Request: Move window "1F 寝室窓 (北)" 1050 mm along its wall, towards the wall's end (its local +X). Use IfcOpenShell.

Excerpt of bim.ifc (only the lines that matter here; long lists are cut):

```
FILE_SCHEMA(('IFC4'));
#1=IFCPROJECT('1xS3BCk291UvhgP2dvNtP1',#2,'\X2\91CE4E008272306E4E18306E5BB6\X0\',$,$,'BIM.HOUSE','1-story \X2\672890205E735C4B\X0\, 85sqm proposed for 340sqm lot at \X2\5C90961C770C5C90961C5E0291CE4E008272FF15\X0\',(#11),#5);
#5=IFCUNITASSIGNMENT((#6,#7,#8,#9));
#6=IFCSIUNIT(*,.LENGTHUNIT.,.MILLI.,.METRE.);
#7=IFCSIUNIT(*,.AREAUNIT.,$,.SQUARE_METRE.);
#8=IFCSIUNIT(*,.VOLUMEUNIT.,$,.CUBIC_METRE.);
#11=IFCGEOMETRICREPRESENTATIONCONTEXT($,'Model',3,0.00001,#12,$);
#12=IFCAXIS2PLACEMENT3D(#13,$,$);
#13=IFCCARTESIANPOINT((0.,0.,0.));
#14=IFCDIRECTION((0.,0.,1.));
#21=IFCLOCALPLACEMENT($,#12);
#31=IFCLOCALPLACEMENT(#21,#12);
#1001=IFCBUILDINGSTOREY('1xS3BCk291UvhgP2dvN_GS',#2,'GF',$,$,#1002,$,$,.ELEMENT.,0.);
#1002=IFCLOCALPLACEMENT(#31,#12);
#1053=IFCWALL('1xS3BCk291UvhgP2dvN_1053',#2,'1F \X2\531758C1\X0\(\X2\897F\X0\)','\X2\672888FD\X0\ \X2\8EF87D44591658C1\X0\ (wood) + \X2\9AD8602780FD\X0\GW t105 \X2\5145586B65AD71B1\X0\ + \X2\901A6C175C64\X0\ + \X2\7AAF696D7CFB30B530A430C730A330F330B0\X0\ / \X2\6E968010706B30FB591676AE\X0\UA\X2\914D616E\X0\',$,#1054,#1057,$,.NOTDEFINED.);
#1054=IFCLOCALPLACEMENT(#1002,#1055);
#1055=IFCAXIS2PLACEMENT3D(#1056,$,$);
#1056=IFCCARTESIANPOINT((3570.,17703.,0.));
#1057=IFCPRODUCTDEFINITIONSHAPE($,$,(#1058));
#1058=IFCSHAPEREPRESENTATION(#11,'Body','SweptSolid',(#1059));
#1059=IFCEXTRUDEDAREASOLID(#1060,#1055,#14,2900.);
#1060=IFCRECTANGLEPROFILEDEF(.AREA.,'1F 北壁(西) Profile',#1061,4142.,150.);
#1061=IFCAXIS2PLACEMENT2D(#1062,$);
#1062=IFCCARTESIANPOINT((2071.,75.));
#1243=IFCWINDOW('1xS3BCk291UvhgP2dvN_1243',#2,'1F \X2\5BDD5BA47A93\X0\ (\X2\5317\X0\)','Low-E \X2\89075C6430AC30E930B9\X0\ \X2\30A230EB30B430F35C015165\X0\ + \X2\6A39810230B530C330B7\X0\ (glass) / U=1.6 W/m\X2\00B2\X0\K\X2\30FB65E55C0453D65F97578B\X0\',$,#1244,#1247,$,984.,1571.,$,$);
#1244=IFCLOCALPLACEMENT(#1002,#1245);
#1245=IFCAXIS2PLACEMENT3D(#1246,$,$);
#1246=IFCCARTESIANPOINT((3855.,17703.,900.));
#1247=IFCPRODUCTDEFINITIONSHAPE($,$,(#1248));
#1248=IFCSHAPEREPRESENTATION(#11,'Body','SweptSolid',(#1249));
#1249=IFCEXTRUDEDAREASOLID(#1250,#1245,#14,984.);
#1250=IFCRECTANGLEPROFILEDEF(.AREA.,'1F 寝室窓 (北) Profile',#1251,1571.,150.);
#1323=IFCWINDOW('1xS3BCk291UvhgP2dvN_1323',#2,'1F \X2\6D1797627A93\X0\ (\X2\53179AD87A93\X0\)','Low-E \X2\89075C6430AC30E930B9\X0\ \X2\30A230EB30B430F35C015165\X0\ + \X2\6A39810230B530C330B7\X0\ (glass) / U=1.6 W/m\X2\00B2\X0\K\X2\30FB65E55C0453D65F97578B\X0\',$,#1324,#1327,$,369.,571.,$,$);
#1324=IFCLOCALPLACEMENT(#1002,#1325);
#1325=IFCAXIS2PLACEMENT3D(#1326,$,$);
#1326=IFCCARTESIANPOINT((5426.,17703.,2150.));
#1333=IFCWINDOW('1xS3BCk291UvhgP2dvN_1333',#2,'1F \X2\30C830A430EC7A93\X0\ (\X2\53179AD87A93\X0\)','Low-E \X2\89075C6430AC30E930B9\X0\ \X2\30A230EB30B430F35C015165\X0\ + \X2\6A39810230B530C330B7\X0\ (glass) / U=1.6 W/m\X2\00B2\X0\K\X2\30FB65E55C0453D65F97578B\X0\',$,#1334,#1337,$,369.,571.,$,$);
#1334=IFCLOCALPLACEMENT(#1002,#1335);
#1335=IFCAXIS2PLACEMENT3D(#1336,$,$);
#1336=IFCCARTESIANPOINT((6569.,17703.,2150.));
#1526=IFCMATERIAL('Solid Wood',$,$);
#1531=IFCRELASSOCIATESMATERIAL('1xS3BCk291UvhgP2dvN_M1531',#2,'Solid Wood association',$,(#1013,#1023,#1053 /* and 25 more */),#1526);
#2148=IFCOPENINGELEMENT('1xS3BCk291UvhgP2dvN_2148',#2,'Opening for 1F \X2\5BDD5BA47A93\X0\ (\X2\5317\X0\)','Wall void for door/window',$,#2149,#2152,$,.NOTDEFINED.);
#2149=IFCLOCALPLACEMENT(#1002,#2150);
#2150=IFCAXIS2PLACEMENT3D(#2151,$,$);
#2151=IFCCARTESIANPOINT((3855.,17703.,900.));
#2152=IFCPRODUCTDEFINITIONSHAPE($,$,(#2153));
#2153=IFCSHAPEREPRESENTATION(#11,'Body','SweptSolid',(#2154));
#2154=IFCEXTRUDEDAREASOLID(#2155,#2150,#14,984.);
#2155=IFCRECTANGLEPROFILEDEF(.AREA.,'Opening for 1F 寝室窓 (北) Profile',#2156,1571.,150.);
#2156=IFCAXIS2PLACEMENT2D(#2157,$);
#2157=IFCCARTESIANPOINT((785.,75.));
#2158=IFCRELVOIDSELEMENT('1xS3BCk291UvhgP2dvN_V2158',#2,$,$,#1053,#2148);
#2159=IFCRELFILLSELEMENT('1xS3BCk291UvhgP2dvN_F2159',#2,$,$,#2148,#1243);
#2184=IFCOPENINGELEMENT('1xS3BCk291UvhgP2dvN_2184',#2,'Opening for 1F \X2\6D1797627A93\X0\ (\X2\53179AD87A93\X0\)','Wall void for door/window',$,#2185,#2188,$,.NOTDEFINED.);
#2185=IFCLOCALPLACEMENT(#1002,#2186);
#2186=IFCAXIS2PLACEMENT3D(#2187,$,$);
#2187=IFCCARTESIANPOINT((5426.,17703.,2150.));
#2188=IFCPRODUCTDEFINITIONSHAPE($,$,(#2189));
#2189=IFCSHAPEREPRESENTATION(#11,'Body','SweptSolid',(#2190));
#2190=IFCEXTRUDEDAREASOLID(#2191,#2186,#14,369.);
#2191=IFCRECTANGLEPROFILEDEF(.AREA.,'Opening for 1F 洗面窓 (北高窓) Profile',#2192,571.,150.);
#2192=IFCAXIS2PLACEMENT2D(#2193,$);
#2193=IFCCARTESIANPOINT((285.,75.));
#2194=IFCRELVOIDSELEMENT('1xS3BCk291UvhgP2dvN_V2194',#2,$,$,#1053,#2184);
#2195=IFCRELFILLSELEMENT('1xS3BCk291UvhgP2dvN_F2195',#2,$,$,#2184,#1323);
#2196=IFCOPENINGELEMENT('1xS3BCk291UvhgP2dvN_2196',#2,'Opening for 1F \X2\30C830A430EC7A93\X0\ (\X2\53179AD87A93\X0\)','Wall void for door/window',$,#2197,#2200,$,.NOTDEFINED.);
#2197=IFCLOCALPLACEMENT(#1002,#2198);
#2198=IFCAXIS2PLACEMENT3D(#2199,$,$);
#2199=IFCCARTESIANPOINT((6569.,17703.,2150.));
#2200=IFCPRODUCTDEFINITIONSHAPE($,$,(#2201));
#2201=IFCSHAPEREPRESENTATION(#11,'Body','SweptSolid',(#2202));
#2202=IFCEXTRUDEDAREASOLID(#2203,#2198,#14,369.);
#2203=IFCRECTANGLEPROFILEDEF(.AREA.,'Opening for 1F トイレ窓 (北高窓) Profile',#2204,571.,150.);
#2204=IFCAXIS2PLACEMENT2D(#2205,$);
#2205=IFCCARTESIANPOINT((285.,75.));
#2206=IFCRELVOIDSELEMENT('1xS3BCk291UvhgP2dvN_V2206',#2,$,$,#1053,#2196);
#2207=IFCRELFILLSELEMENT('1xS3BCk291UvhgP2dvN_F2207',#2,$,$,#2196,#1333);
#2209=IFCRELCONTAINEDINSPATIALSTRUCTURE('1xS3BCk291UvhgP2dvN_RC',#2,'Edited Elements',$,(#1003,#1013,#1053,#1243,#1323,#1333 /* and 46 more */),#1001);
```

```python
import ifcopenshell
import ifcopenshell.api.geometry
import ifcopenshell.util.placement
import ifcopenshell.util.unit

model = ifcopenshell.open("bim.ifc")
unit_scale = ifcopenshell.util.unit.calculate_unit_scale(model)

window = model.by_id(1243)
opening = window.FillsVoids[0].RelatingOpeningElement
wall = opening.VoidsElements[0].RelatingBuildingElement

wall_matrix = ifcopenshell.util.placement.get_local_placement(wall.ObjectPlacement)
shift = wall_matrix[:3, 0] * 1.05 / unit_scale
before = ifcopenshell.util.placement.get_local_placement(window.ObjectPlacement)[:3, 3].copy()

# The window is not placed relative to its opening, so move both.
for product in (opening, window):
    matrix = ifcopenshell.util.placement.get_local_placement(product.ObjectPlacement)
    matrix[:3, 3] += shift
    ifcopenshell.api.geometry.edit_object_placement(model, product=product, matrix=matrix, is_si=False)

after = ifcopenshell.util.placement.get_local_placement(window.ObjectPlacement)[:3, 3]
print("window moved by", (after - before).round(3) + 0.0)

model.write("bim_v2.ifc")
```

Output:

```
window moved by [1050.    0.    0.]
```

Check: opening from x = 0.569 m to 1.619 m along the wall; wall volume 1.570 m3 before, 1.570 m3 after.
